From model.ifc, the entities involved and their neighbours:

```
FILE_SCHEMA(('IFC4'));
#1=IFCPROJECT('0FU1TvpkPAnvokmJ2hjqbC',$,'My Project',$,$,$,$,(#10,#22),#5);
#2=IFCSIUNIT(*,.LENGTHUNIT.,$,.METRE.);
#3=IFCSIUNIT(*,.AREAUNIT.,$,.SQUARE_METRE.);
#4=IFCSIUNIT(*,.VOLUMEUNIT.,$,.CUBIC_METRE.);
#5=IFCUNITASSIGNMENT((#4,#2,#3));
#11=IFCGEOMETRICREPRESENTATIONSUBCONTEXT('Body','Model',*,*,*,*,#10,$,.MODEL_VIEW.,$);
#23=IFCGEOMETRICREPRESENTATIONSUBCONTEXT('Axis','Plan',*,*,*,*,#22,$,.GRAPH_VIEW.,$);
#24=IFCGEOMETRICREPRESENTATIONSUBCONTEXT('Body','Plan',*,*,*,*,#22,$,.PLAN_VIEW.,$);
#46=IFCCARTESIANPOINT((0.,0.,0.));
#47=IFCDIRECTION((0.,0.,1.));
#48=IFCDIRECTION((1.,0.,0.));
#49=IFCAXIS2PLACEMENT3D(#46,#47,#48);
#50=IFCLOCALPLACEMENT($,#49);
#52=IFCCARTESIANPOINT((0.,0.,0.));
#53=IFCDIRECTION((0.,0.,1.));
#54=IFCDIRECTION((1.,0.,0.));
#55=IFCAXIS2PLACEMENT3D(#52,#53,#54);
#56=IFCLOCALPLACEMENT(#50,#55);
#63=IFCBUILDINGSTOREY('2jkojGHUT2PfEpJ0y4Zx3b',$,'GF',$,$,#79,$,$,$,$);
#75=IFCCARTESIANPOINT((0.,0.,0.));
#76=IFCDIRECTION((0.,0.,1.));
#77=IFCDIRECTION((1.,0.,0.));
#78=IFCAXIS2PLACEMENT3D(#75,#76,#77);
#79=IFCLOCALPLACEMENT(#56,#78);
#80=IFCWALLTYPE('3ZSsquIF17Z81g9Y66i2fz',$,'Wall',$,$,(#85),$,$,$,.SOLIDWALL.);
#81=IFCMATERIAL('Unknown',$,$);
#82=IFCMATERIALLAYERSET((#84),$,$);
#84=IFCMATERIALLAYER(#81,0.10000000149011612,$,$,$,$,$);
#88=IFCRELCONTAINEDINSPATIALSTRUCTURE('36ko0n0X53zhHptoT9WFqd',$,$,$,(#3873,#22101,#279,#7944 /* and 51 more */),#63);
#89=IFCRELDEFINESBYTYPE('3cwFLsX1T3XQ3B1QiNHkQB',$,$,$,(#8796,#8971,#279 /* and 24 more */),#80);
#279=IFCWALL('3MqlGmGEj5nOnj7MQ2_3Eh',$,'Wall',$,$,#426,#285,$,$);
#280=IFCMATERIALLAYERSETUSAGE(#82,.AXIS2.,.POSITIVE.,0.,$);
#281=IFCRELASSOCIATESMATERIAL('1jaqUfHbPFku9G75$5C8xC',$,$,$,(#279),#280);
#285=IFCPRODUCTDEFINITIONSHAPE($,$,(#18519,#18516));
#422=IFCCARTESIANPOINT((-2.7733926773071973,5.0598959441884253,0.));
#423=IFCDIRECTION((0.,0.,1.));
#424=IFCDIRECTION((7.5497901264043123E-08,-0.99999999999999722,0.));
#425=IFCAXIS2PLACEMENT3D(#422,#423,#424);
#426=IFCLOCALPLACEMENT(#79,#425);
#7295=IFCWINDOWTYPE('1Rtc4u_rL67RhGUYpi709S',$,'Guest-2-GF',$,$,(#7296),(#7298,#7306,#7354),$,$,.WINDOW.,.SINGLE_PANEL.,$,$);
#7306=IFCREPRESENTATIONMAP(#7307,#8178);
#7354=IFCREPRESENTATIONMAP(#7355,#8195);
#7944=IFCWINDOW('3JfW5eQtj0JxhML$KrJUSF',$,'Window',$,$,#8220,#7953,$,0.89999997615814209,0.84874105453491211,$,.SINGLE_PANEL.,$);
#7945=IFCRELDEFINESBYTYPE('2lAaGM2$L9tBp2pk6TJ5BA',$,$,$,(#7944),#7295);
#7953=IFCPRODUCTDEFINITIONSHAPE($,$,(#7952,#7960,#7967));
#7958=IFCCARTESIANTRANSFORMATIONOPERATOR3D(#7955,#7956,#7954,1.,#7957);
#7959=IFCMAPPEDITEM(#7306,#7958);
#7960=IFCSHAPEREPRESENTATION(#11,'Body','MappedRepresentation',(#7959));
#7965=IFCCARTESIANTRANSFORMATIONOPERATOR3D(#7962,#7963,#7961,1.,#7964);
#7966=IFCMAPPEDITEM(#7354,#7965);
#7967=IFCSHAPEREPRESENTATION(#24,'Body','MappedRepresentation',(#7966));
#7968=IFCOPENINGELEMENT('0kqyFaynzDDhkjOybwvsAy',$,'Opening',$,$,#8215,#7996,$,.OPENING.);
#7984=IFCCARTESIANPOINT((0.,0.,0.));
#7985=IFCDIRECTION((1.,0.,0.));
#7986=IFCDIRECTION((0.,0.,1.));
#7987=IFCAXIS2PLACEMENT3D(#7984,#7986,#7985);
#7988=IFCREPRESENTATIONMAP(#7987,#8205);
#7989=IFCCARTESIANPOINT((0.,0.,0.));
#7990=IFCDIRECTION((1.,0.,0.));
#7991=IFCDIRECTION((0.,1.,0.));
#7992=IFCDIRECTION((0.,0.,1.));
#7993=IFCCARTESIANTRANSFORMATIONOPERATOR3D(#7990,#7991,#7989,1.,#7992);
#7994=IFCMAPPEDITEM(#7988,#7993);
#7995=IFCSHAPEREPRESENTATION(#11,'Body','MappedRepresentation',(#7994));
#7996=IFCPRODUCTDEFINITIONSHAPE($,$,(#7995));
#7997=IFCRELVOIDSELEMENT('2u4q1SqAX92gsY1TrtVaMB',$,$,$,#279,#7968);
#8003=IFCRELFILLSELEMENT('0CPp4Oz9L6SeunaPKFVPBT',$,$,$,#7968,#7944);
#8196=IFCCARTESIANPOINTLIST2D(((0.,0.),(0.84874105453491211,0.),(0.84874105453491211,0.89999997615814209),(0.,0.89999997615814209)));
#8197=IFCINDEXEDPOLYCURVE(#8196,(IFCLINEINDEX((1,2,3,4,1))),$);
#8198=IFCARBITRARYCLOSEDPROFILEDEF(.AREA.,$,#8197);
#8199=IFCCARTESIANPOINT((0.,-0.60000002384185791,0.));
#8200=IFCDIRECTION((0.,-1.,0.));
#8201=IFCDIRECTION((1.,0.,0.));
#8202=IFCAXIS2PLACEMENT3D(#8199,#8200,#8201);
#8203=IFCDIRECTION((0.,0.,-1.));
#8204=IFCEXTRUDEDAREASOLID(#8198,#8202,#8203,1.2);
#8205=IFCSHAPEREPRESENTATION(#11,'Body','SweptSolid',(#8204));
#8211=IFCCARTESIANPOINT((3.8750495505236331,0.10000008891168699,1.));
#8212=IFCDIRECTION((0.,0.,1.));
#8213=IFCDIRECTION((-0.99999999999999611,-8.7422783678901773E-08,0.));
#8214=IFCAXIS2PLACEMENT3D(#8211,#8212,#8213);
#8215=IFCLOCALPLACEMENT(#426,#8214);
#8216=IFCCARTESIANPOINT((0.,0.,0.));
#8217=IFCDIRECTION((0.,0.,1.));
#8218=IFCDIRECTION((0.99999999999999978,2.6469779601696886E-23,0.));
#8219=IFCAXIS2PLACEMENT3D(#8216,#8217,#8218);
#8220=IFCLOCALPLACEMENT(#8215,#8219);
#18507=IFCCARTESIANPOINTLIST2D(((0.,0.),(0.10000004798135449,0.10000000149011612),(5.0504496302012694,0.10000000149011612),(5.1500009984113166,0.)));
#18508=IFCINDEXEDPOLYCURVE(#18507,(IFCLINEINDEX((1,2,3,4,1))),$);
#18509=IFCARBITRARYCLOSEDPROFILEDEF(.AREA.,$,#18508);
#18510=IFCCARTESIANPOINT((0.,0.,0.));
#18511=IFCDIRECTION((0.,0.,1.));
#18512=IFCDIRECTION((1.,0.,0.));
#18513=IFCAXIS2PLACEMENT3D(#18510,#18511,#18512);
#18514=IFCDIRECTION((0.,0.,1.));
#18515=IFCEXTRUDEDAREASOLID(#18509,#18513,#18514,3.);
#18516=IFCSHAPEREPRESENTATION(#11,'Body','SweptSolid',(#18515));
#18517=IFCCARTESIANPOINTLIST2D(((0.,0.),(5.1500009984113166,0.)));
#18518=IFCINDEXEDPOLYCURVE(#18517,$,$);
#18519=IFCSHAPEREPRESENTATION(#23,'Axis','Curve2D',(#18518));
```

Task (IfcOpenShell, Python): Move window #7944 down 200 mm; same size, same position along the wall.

```python
import numpy as np
import ifcopenshell
import ifcopenshell.api.geometry
import ifcopenshell.util.placement
import ifcopenshell.util.unit

model = ifcopenshell.open("model.ifc")
unit_scale = ifcopenshell.util.unit.calculate_unit_scale(model)

window = model.by_id(7944)
opening = window.FillsVoids[0].RelatingOpeningElement
dz = -0.2 / unit_scale

shift = np.array([0.0, 0.0, dz])
# The window is placed relative to its opening, so it follows when the opening moves.
matrix = ifcopenshell.util.placement.get_local_placement(opening.ObjectPlacement)
matrix[:3, 3] += shift
ifcopenshell.api.geometry.edit_object_placement(
    model, product=opening, matrix=matrix, is_si=False, should_transform_children=True
)

print(f"moved by {dz * unit_scale:+.3f} m")

model.write("model_edited.ifc")
```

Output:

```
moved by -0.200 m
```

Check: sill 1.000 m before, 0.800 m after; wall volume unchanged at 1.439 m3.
